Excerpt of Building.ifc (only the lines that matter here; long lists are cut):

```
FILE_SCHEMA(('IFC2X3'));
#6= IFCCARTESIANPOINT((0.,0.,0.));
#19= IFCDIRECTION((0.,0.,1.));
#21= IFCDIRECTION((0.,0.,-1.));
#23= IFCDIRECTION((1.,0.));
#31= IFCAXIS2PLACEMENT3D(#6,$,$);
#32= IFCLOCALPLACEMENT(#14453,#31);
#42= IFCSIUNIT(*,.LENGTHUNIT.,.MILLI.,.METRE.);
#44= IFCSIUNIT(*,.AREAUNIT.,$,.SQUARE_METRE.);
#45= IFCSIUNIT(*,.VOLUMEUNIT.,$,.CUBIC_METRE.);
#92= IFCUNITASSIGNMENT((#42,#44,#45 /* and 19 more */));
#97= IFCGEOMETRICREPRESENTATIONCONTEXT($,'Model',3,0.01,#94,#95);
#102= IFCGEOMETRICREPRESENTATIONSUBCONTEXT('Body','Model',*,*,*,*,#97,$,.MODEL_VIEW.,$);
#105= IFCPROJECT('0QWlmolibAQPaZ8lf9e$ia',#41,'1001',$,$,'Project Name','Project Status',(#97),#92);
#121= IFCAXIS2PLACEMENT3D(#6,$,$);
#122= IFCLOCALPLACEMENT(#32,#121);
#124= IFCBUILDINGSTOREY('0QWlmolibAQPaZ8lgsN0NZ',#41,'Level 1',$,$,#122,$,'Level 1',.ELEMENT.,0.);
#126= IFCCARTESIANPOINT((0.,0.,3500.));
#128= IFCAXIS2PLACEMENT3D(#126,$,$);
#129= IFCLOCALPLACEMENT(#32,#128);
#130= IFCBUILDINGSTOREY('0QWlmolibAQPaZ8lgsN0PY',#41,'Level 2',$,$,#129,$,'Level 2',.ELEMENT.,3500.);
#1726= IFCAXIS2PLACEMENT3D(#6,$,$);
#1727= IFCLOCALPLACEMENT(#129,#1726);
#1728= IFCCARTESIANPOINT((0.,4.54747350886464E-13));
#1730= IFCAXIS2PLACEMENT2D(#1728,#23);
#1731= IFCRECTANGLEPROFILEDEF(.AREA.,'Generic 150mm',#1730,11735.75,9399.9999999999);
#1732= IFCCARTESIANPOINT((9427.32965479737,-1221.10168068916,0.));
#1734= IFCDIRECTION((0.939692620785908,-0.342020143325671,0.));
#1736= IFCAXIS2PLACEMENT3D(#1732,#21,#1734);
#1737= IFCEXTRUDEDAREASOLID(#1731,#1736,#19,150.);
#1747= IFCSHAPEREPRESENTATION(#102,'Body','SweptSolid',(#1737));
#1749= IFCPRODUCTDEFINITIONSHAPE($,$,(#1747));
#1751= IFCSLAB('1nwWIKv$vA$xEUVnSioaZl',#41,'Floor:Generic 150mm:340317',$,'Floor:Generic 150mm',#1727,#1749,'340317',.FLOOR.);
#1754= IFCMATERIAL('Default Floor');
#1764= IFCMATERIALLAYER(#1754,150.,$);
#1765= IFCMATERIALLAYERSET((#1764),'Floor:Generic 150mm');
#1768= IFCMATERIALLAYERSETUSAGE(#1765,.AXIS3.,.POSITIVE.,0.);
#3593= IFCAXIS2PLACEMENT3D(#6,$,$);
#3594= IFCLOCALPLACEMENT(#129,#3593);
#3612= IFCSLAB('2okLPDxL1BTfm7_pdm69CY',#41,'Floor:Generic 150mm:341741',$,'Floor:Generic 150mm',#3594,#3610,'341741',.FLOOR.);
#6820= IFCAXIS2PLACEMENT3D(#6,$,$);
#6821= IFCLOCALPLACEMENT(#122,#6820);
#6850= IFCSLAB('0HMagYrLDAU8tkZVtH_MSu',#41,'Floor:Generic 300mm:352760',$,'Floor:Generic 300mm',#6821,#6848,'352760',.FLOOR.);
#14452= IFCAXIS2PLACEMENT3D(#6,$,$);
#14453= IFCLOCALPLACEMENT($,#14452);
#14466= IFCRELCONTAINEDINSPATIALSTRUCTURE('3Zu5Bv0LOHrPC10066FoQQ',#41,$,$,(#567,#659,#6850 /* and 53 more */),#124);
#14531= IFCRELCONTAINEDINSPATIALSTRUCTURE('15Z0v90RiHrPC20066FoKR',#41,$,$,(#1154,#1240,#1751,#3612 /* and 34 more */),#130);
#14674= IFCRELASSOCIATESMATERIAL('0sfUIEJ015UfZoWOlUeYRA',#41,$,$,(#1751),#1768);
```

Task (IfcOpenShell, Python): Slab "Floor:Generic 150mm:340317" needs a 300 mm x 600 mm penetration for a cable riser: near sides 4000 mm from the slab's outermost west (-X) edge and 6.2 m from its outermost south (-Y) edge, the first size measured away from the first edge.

```python
import numpy as np
import ifcopenshell
import ifcopenshell.api.feature
import ifcopenshell.api.geometry
import ifcopenshell.api.root
import ifcopenshell.geom
import ifcopenshell.util.placement
import ifcopenshell.util.representation
import ifcopenshell.util.shape
import ifcopenshell.util.unit

model = ifcopenshell.open("Building.ifc")
unit_scale = ifcopenshell.util.unit.calculate_unit_scale(model)
settings = ifcopenshell.geom.settings()


def volume(element):
    """Net volume in cubic metres, openings subtracted."""
    shape = ifcopenshell.geom.create_shape(settings, element)
    return ifcopenshell.util.shape.get_volume(shape.geometry)


slab = model.by_guid("1nwWIKv$vA$xEUVnSioaZl")
before = volume(slab)

# Extent in the slab's own axes, in metres. The edges named are its -X and -Y sides.
slab_shape = ifcopenshell.geom.create_shape(settings, slab)
vertices = ifcopenshell.util.shape.get_vertices(slab_shape.geometry)
x_min, y_min, bottom = vertices.min(axis=0)
top = vertices[:, 2].max()

opening = ifcopenshell.api.root.create_entity(model, ifc_class="IfcOpeningElement", name="Cable riser opening")
context = ifcopenshell.util.representation.get_context(model, "Model", "Body", "MODEL_VIEW")
width, depth = 0.3, 0.6
outline = [(0.0, 0.0), (width, 0.0), (width, depth), (0.0, depth), (0.0, 0.0)]
# Overshoot both faces by 50 mm so the cut is clean.
shape = ifcopenshell.api.geometry.add_slab_representation(
    model, context=context, depth=top - bottom + 0.1, polyline=outline
)
ifcopenshell.api.geometry.assign_representation(model, product=opening, representation=shape)

matrix = ifcopenshell.util.placement.get_local_placement(slab.ObjectPlacement)
matrix[:, 3] = matrix @ np.append(np.array([x_min + 4, y_min + 6.2, bottom - 0.05]) / unit_scale, 1.0)
ifcopenshell.api.geometry.edit_object_placement(model, product=opening, matrix=matrix, is_si=False)
ifcopenshell.api.feature.add_feature(model, feature=opening, element=slab)

after = volume(slab)

print(f"slab volume {before:.3f} -> {after:.3f} m3")

model.write("Building-out.ifc")
```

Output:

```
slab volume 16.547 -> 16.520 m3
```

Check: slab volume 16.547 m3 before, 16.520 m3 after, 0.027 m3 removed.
